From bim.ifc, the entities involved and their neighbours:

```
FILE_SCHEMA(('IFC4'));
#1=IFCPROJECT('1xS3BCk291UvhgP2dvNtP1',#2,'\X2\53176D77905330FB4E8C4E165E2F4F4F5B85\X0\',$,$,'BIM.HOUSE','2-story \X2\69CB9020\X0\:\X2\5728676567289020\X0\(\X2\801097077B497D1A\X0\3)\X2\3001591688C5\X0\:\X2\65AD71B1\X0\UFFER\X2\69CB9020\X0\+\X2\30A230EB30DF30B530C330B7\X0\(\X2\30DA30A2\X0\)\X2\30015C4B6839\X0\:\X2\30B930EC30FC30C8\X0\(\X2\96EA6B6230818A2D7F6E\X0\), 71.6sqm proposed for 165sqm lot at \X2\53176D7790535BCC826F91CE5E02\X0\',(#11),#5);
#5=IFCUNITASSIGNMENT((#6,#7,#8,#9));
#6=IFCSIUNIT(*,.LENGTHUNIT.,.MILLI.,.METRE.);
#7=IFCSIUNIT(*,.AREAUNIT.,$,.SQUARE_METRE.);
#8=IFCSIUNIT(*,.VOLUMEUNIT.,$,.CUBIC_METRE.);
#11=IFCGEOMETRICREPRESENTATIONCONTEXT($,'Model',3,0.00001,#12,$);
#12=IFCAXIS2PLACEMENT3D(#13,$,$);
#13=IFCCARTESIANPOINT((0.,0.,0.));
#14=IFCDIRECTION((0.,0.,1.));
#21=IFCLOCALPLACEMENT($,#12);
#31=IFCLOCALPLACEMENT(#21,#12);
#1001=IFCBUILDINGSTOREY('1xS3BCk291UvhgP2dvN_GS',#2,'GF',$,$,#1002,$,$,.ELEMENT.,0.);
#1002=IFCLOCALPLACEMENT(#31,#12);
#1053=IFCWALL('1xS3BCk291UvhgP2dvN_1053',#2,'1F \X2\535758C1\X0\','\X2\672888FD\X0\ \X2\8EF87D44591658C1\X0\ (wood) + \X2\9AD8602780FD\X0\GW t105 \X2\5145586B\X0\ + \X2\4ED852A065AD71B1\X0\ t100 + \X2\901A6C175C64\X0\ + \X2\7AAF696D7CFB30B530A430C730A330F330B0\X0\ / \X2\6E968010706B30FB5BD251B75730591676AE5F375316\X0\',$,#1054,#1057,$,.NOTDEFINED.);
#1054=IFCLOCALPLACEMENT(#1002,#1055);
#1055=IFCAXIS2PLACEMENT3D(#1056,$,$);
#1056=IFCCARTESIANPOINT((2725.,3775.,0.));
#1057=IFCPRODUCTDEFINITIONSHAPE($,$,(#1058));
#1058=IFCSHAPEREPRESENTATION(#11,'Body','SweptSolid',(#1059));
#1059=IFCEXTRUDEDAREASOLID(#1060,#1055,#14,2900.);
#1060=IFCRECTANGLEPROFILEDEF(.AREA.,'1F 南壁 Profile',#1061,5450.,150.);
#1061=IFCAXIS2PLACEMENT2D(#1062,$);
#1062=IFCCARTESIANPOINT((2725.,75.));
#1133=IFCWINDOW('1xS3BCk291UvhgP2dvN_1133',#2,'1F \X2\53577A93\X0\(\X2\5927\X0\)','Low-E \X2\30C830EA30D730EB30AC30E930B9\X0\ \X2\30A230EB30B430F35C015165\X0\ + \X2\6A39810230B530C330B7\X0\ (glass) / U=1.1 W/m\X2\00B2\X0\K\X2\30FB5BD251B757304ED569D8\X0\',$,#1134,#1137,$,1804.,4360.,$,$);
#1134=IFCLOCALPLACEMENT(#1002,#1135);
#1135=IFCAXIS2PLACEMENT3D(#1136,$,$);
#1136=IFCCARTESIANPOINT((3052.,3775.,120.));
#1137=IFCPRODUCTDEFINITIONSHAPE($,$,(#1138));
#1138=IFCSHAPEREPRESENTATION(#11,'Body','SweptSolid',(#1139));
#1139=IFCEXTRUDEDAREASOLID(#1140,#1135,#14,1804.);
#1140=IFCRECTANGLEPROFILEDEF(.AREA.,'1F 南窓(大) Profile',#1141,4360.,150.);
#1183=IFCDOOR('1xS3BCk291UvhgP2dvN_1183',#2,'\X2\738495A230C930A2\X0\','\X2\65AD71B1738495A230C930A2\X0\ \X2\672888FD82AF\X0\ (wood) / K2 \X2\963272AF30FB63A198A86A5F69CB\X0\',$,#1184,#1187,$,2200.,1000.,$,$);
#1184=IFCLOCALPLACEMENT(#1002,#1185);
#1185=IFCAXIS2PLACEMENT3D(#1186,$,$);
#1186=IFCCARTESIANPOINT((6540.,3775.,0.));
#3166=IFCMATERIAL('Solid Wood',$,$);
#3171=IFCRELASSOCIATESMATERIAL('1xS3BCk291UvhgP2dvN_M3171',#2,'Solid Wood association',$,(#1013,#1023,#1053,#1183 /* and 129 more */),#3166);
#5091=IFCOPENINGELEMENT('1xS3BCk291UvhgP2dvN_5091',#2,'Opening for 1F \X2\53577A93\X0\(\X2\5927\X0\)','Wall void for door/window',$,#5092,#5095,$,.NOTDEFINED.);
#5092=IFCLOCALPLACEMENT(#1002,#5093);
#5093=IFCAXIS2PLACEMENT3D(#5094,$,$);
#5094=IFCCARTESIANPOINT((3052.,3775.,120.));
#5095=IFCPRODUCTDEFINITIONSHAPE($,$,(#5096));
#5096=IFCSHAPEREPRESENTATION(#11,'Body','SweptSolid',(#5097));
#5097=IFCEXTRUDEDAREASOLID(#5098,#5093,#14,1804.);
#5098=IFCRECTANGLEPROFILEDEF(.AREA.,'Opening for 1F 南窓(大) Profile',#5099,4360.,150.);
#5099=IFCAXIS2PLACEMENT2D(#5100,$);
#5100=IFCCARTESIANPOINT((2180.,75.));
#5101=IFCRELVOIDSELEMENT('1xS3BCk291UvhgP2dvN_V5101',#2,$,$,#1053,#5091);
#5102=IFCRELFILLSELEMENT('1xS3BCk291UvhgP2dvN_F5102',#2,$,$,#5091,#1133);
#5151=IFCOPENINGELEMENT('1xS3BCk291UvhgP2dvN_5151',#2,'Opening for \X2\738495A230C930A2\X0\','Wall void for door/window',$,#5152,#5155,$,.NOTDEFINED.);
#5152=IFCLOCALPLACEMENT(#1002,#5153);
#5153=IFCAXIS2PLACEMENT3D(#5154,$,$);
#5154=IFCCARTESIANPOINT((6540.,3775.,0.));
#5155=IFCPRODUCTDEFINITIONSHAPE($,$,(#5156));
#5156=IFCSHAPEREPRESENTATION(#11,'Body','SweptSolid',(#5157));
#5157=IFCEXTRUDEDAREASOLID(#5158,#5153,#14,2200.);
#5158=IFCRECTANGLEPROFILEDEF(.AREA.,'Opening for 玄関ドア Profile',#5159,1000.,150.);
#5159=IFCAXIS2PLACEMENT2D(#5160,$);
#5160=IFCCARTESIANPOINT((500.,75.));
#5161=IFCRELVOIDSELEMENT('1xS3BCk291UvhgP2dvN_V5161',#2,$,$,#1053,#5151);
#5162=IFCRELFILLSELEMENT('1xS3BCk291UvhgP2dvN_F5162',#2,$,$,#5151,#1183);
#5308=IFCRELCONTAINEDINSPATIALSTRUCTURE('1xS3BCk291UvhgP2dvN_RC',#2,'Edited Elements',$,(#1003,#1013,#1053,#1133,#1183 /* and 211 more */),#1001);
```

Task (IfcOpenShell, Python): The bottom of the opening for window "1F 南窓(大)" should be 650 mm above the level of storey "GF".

```python
import numpy as np
import ifcopenshell
import ifcopenshell.api.geometry
import ifcopenshell.geom
import ifcopenshell.util.element
import ifcopenshell.util.placement
import ifcopenshell.util.shape
import ifcopenshell.util.unit

model = ifcopenshell.open("bim.ifc")
unit_scale = ifcopenshell.util.unit.calculate_unit_scale(model)

window = model.by_id(1133)
opening = window.FillsVoids[0].RelatingOpeningElement
storey = ifcopenshell.util.element.get_container(window, ifc_class="IfcBuildingStorey")
level = ifcopenshell.util.placement.get_local_placement(storey.ObjectPlacement)[2, 3]

# The opening's origin need not be at the sill, so measure its lowest point.
shape = ifcopenshell.geom.create_shape(ifcopenshell.geom.settings(), opening)
bottom = ifcopenshell.util.shape.get_shape_bottom_elevation(shape, shape.geometry) / unit_scale
dz = level + 650.0 - bottom

shift = np.array([0.0, 0.0, dz])
# The window is not placed relative to its opening, so move both.
for product in (opening, window):
    matrix = ifcopenshell.util.placement.get_local_placement(product.ObjectPlacement)
    matrix[:3, 3] += shift
    ifcopenshell.api.geometry.edit_object_placement(model, product=product, matrix=matrix, is_si=False)

print(f"moved by {dz * unit_scale:+.3f} m")

model.write("bim_edited.ifc")
```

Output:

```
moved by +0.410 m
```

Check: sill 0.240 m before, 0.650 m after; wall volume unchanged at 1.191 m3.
